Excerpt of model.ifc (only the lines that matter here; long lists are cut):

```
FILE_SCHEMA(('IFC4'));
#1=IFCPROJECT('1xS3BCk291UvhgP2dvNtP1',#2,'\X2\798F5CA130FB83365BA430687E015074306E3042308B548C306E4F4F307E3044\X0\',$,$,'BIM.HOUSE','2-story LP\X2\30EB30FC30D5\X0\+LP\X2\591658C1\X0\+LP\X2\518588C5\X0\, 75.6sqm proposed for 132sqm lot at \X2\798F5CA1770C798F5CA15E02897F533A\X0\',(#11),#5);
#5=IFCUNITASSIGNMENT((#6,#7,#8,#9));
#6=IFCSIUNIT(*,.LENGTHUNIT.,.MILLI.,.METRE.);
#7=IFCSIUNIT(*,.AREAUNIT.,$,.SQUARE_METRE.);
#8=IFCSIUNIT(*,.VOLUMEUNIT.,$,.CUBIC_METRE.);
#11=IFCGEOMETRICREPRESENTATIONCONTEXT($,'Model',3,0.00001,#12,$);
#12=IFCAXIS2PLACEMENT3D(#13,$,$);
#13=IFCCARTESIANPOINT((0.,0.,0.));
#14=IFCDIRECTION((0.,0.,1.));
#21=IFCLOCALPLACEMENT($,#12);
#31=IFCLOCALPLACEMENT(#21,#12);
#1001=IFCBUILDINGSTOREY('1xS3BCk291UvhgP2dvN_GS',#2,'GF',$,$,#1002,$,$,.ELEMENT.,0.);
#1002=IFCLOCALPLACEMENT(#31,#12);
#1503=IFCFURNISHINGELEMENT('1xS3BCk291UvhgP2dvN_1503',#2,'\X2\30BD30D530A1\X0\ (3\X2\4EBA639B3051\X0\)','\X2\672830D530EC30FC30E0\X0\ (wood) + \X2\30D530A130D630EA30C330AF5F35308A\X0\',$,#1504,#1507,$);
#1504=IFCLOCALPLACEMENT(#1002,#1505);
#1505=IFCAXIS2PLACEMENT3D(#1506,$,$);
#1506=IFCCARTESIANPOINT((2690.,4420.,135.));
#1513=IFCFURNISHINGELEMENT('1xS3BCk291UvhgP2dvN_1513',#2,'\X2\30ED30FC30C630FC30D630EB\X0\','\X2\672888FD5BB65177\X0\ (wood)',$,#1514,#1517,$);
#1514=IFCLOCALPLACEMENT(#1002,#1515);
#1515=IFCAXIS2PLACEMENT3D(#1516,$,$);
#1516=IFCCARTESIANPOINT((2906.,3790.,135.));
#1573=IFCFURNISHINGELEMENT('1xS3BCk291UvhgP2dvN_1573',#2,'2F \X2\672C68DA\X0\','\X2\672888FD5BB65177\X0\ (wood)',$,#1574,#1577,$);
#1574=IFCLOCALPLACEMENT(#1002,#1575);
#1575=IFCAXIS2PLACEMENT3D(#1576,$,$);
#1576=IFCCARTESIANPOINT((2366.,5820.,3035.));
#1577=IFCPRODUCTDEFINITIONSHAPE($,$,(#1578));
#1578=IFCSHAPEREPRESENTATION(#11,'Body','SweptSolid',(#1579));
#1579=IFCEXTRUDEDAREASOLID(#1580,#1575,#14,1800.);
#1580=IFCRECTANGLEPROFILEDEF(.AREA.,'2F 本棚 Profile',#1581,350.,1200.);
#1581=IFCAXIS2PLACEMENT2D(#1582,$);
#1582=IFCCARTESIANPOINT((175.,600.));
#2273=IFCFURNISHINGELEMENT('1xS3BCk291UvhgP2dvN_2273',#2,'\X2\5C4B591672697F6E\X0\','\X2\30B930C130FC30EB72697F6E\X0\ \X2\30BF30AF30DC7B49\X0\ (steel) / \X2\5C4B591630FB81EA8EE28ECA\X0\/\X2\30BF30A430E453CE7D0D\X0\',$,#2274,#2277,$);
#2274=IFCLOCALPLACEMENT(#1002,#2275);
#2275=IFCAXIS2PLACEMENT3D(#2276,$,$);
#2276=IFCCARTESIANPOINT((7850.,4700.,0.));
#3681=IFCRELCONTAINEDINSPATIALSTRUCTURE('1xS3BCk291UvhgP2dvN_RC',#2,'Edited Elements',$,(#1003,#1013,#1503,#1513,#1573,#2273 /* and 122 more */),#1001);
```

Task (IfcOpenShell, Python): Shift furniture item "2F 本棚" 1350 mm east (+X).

```python
import ifcopenshell
import ifcopenshell.api.geometry
import ifcopenshell.util.placement
import ifcopenshell.util.unit

model = ifcopenshell.open("model.ifc")
unit_scale = ifcopenshell.util.unit.calculate_unit_scale(model)

item = model.by_guid("1xS3BCk291UvhgP2dvN_1573")
matrix = ifcopenshell.util.placement.get_local_placement(item.ObjectPlacement)
matrix[0, 3] += 1.35 / unit_scale
ifcopenshell.api.geometry.edit_object_placement(model, product=item, matrix=matrix, is_si=False)

print(ifcopenshell.util.placement.get_local_placement(item.ObjectPlacement).round(3) + 0.0)

model.write("model_rev.ifc")
```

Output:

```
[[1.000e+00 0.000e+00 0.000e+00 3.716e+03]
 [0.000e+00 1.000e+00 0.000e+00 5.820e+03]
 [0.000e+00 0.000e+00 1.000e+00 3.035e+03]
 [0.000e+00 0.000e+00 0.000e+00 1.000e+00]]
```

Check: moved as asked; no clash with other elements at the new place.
